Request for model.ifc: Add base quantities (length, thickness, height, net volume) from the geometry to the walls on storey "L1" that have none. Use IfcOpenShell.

First a look at what the model holds.

```python
import ifcopenshell
import ifcopenshell.util.element
import ifcopenshell.util.unit

model = ifcopenshell.open("model.ifc")
print(model.schema)
for unit_type in ("LENGTHUNIT", "AREAUNIT", "VOLUMEUNIT"):
    print(unit_type, ifcopenshell.util.unit.calculate_unit_scale(model, unit_type))
storey = next(s for s in model.by_type("IfcBuildingStorey") if s.Name == "L1")
walls = [e for e in ifcopenshell.util.element.get_decomposition(storey) if e.is_a("IfcWall")]
for e in sorted(walls, key=lambda e: e.id()):
    print(e.id(), e.is_a(), e.Name, list(ifcopenshell.util.element.get_psets(e, qtos_only=True)), sep=" | ")
```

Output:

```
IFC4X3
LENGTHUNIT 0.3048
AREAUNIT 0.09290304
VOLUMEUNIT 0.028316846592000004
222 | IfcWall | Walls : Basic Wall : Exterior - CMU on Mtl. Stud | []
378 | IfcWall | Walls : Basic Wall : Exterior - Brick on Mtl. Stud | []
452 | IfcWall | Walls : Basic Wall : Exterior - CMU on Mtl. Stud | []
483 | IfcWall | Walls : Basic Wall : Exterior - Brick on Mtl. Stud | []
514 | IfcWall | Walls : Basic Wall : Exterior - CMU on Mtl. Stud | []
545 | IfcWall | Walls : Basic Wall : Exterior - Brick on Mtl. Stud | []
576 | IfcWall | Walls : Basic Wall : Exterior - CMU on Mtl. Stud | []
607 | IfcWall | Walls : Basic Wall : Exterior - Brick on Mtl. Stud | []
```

```python
import ifcopenshell
import ifcopenshell.api.pset
import ifcopenshell.geom
import ifcopenshell.util.element
import ifcopenshell.util.shape
import ifcopenshell.util.unit

model = ifcopenshell.open("model.ifc")
unit_scale = ifcopenshell.util.unit.calculate_unit_scale(model)
volume_scale = ifcopenshell.util.unit.calculate_unit_scale(model, "VOLUMEUNIT")
settings = ifcopenshell.geom.settings()

storey = next(s for s in model.by_type("IfcBuildingStorey") if s.Name == "L1")
walls = [e for e in ifcopenshell.util.element.get_decomposition(storey) if e.is_a("IfcWall")]

for e in sorted(walls, key=lambda e: e.id()):
    if ifcopenshell.util.element.get_psets(e, qtos_only=True, should_inherit=False):
        continue
    # Geometry comes back in metres, in the element's own axes.
    shape = ifcopenshell.geom.create_shape(settings, e)
    values = {
        "Length": ifcopenshell.util.shape.get_x(shape.geometry) / unit_scale,
        "Width": ifcopenshell.util.shape.get_y(shape.geometry) / unit_scale,
        "Height": ifcopenshell.util.shape.get_z(shape.geometry) / unit_scale,
        "NetVolume": ifcopenshell.util.shape.get_volume(shape.geometry) / volume_scale,
    }
    qto = ifcopenshell.api.pset.add_qto(model, product=e, name="Qto_WallBaseQuantities")
    ifcopenshell.api.pset.edit_qto(model, qto=qto, properties=values)
    print(e.id(), {k: round(v, 3) for k, v in values.items()})

model.write("model_updated.ifc")
```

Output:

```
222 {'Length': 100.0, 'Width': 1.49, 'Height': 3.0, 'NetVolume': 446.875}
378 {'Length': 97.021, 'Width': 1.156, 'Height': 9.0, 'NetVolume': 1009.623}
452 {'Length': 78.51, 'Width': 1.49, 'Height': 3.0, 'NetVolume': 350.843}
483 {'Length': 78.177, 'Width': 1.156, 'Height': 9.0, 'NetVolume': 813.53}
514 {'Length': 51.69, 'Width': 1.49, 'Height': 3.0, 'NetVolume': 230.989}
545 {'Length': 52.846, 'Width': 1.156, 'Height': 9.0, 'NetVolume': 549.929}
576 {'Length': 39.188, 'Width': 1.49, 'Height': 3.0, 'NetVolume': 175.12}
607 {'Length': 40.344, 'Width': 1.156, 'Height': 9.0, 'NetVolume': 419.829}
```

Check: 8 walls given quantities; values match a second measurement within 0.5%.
